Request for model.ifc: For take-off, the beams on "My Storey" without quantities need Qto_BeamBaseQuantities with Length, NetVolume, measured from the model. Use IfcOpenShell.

First a look at what the model holds.

```python
import ifcopenshell
import ifcopenshell.util.element
import ifcopenshell.util.unit

model = ifcopenshell.open("model.ifc")
print(model.schema)
for unit_type in ("LENGTHUNIT", "AREAUNIT", "VOLUMEUNIT"):
    print(unit_type, ifcopenshell.util.unit.calculate_unit_scale(model, unit_type))
storey = next(s for s in model.by_type("IfcBuildingStorey") if s.Name == "My Storey")
beams = [e for e in ifcopenshell.util.element.get_decomposition(storey) if e.is_a("IfcBeam")]
for e in sorted(beams, key=lambda e: e.id()):
    print(e.id(), e.is_a(), e.Name, list(ifcopenshell.util.element.get_psets(e, qtos_only=True)), sep=" | ")
```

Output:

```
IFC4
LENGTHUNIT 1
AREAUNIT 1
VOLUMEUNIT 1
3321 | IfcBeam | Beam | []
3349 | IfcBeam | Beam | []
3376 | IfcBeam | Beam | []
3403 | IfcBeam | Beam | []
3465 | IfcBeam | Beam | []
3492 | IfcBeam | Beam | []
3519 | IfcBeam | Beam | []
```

```python
import ifcopenshell
import ifcopenshell.api.pset
import ifcopenshell.geom
import ifcopenshell.util.element
import ifcopenshell.util.shape
import ifcopenshell.util.unit

model = ifcopenshell.open("model.ifc")
unit_scale = ifcopenshell.util.unit.calculate_unit_scale(model)
volume_scale = ifcopenshell.util.unit.calculate_unit_scale(model, "VOLUMEUNIT")
settings = ifcopenshell.geom.settings()

storey = next(s for s in model.by_type("IfcBuildingStorey") if s.Name == "My Storey")
beams = [e for e in ifcopenshell.util.element.get_decomposition(storey) if e.is_a("IfcBeam")]

for e in sorted(beams, key=lambda e: e.id()):
    if ifcopenshell.util.element.get_psets(e, qtos_only=True, should_inherit=False):
        continue
    # Geometry comes back in metres, in the element's own axes.
    shape = ifcopenshell.geom.create_shape(settings, e)
    values = {
        "Length": ifcopenshell.util.shape.get_max_xyz(shape.geometry) / unit_scale,
        "NetVolume": ifcopenshell.util.shape.get_volume(shape.geometry) / volume_scale,
    }
    qto = ifcopenshell.api.pset.add_qto(model, product=e, name="Qto_BeamBaseQuantities")
    ifcopenshell.api.pset.edit_qto(model, qto=qto, properties=values)
    print(e.id(), {k: round(v, 3) for k, v in values.items()})

model.write("model-out.ifc")
```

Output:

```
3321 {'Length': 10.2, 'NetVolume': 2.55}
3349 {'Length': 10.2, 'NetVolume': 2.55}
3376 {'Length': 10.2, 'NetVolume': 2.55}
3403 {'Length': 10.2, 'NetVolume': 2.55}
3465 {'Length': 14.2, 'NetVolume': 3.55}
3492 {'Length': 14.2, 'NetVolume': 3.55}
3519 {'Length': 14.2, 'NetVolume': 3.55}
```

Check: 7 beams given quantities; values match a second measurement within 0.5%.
